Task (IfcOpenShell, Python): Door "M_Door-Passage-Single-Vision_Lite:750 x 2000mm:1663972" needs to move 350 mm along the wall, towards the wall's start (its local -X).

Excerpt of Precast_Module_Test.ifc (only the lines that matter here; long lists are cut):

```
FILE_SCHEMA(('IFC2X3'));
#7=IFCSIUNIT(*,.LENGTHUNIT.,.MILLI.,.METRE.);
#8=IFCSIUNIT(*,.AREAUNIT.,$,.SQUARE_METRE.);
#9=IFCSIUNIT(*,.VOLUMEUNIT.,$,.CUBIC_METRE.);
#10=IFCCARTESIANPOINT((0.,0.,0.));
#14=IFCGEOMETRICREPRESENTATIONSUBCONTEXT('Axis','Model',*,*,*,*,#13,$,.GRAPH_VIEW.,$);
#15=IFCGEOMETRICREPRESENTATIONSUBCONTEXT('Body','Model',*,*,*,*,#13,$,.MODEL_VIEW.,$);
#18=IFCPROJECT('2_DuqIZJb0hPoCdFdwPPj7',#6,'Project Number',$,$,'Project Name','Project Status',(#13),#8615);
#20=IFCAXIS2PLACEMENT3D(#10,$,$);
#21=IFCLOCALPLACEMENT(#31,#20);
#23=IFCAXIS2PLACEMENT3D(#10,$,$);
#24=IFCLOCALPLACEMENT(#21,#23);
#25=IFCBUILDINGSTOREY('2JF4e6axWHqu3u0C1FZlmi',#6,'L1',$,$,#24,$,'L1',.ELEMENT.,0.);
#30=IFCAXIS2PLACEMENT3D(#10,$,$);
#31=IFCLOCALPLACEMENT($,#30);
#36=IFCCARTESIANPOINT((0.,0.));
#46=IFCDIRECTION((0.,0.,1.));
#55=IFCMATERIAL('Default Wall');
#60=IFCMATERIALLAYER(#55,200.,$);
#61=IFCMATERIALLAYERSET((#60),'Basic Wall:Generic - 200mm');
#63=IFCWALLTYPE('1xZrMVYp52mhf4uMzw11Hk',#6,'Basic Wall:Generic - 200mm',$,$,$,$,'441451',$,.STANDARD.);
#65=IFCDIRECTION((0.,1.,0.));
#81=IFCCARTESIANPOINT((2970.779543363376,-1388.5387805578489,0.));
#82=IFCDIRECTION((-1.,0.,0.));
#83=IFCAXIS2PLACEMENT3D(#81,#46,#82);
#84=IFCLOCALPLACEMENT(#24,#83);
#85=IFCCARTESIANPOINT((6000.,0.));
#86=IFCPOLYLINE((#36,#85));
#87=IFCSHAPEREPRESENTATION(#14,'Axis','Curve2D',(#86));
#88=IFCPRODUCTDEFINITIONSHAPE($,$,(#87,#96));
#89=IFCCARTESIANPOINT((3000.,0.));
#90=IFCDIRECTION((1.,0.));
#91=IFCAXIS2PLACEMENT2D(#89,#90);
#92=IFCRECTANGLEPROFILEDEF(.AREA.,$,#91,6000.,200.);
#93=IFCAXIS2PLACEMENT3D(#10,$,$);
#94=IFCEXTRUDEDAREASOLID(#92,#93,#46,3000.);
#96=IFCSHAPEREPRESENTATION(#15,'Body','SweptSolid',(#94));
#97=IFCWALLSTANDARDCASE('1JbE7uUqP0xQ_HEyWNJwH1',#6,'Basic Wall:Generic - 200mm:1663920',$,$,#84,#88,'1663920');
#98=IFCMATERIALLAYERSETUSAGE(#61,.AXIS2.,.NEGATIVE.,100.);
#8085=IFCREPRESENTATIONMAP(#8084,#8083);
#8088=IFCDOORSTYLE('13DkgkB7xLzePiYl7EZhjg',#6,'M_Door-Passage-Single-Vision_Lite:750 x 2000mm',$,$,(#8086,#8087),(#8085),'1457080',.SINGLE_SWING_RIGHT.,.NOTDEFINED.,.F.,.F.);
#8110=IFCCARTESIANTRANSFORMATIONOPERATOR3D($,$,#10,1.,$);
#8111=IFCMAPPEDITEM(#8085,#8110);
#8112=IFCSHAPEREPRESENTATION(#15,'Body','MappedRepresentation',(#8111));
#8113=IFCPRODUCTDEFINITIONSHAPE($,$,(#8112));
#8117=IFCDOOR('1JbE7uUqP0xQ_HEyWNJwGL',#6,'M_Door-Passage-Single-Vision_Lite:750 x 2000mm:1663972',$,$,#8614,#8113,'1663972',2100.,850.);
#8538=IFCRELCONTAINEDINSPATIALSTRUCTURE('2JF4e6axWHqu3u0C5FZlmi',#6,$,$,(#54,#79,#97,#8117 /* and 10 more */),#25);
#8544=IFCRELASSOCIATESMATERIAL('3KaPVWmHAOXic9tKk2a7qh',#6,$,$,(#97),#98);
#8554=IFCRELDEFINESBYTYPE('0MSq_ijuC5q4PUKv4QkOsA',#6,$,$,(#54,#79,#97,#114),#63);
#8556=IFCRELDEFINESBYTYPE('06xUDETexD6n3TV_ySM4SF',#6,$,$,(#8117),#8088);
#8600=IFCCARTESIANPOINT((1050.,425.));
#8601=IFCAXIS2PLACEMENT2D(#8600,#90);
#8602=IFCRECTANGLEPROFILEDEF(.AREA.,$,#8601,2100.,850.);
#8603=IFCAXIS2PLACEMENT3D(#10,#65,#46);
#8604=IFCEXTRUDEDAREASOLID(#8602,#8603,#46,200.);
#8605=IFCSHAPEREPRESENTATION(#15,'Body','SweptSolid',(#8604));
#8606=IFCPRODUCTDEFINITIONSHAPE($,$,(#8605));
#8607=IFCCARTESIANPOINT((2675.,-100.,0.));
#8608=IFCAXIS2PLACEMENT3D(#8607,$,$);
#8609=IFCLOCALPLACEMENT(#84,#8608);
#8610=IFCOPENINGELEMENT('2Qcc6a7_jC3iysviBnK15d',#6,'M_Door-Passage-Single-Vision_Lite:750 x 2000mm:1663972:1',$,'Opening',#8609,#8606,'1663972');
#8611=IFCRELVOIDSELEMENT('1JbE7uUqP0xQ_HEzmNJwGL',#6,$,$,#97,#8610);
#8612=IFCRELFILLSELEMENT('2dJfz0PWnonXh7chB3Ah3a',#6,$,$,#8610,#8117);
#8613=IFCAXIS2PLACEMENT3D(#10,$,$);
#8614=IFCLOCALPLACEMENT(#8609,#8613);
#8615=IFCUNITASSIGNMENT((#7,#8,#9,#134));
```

```python
import ifcopenshell
import ifcopenshell.api.geometry
import ifcopenshell.util.placement
import ifcopenshell.util.unit

model = ifcopenshell.open("Precast_Module_Test.ifc")
unit_scale = ifcopenshell.util.unit.calculate_unit_scale(model)

door = model.by_guid("1JbE7uUqP0xQ_HEyWNJwGL")
opening = door.FillsVoids[0].RelatingOpeningElement
wall = opening.VoidsElements[0].RelatingBuildingElement

wall_matrix = ifcopenshell.util.placement.get_local_placement(wall.ObjectPlacement)
shift = wall_matrix[:3, 0] * -0.35 / unit_scale
before = ifcopenshell.util.placement.get_local_placement(door.ObjectPlacement)[:3, 3].copy()

# The door is placed relative to its opening, so it follows when the opening moves.
matrix = ifcopenshell.util.placement.get_local_placement(opening.ObjectPlacement)
matrix[:3, 3] += shift
ifcopenshell.api.geometry.edit_object_placement(
    model, product=opening, matrix=matrix, is_si=False, should_transform_children=True
)

after = ifcopenshell.util.placement.get_local_placement(door.ObjectPlacement)[:3, 3]
print("door moved by", (after - before).round(3) + 0.0)

model.write("Precast_Module_Test_updated.ifc")
```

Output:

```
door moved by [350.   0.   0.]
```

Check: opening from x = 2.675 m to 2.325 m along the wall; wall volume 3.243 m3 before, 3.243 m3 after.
